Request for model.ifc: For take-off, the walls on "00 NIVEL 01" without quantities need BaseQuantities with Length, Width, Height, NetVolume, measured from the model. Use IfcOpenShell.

First a look at what the model holds.

```python
import ifcopenshell
import ifcopenshell.util.element
import ifcopenshell.util.unit

model = ifcopenshell.open("model.ifc")
print(model.schema)
for unit_type in ("LENGTHUNIT", "AREAUNIT", "VOLUMEUNIT"):
    print(unit_type, ifcopenshell.util.unit.calculate_unit_scale(model, unit_type))
storey = next(s for s in model.by_type("IfcBuildingStorey") if s.Name == "00 NIVEL 01")
walls = [e for e in ifcopenshell.util.element.get_decomposition(storey) if e.is_a("IfcWall")]
for e in sorted(walls, key=lambda e: e.id()):
    print(e.id(), e.is_a(), e.Name, list(ifcopenshell.util.element.get_psets(e, qtos_only=True)), sep=" | ")
```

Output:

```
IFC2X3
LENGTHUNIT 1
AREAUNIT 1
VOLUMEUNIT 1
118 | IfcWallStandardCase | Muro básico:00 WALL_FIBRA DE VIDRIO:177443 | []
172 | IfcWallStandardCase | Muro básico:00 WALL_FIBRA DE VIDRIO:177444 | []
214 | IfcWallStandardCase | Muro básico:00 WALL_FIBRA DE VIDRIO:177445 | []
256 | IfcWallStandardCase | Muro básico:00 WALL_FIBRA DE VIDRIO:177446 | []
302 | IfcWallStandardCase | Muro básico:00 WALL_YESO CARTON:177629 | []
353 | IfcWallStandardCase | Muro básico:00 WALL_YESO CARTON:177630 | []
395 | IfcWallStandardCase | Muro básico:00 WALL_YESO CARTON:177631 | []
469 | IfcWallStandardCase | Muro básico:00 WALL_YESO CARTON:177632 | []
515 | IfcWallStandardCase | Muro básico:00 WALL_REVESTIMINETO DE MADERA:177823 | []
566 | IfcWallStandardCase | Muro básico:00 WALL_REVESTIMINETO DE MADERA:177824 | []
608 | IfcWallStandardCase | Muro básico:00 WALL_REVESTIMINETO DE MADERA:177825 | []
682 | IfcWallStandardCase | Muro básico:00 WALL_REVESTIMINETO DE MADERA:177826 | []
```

```python
import ifcopenshell
import ifcopenshell.api.pset
import ifcopenshell.geom
import ifcopenshell.util.element
import ifcopenshell.util.shape
import ifcopenshell.util.unit

model = ifcopenshell.open("model.ifc")
unit_scale = ifcopenshell.util.unit.calculate_unit_scale(model)
volume_scale = ifcopenshell.util.unit.calculate_unit_scale(model, "VOLUMEUNIT")
settings = ifcopenshell.geom.settings()

storey = next(s for s in model.by_type("IfcBuildingStorey") if s.Name == "00 NIVEL 01")
walls = [e for e in ifcopenshell.util.element.get_decomposition(storey) if e.is_a("IfcWall")]

for e in sorted(walls, key=lambda e: e.id()):
    if ifcopenshell.util.element.get_psets(e, qtos_only=True, should_inherit=False):
        continue
    # Geometry comes back in metres, in the element's own axes.
    shape = ifcopenshell.geom.create_shape(settings, e)
    values = {
        "Length": ifcopenshell.util.shape.get_x(shape.geometry) / unit_scale,
        "Width": ifcopenshell.util.shape.get_y(shape.geometry) / unit_scale,
        "Height": ifcopenshell.util.shape.get_z(shape.geometry) / unit_scale,
        "NetVolume": ifcopenshell.util.shape.get_volume(shape.geometry) / volume_scale,
    }
    qto = ifcopenshell.api.pset.add_qto(model, product=e, name="BaseQuantities")
    ifcopenshell.api.pset.edit_qto(model, qto=qto, properties=values)
    print(e.id(), {k: round(v, 3) for k, v in values.items()})

model.write("model_edited.ifc")
```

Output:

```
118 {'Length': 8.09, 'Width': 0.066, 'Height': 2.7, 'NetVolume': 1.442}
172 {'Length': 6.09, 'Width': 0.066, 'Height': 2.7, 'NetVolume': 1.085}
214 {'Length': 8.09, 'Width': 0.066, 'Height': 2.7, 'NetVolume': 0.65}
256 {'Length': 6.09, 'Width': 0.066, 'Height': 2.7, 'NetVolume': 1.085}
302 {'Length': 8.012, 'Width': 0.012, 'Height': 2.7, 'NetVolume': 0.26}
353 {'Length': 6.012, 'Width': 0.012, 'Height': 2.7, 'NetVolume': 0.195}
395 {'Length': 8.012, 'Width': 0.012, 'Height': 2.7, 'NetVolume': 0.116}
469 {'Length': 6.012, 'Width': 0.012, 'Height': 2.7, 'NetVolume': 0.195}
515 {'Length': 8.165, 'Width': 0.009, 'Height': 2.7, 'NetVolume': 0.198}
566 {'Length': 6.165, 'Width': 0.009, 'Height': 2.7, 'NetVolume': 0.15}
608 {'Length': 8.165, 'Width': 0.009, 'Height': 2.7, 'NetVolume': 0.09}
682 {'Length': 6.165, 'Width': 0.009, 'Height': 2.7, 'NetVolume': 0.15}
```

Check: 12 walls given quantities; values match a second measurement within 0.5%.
